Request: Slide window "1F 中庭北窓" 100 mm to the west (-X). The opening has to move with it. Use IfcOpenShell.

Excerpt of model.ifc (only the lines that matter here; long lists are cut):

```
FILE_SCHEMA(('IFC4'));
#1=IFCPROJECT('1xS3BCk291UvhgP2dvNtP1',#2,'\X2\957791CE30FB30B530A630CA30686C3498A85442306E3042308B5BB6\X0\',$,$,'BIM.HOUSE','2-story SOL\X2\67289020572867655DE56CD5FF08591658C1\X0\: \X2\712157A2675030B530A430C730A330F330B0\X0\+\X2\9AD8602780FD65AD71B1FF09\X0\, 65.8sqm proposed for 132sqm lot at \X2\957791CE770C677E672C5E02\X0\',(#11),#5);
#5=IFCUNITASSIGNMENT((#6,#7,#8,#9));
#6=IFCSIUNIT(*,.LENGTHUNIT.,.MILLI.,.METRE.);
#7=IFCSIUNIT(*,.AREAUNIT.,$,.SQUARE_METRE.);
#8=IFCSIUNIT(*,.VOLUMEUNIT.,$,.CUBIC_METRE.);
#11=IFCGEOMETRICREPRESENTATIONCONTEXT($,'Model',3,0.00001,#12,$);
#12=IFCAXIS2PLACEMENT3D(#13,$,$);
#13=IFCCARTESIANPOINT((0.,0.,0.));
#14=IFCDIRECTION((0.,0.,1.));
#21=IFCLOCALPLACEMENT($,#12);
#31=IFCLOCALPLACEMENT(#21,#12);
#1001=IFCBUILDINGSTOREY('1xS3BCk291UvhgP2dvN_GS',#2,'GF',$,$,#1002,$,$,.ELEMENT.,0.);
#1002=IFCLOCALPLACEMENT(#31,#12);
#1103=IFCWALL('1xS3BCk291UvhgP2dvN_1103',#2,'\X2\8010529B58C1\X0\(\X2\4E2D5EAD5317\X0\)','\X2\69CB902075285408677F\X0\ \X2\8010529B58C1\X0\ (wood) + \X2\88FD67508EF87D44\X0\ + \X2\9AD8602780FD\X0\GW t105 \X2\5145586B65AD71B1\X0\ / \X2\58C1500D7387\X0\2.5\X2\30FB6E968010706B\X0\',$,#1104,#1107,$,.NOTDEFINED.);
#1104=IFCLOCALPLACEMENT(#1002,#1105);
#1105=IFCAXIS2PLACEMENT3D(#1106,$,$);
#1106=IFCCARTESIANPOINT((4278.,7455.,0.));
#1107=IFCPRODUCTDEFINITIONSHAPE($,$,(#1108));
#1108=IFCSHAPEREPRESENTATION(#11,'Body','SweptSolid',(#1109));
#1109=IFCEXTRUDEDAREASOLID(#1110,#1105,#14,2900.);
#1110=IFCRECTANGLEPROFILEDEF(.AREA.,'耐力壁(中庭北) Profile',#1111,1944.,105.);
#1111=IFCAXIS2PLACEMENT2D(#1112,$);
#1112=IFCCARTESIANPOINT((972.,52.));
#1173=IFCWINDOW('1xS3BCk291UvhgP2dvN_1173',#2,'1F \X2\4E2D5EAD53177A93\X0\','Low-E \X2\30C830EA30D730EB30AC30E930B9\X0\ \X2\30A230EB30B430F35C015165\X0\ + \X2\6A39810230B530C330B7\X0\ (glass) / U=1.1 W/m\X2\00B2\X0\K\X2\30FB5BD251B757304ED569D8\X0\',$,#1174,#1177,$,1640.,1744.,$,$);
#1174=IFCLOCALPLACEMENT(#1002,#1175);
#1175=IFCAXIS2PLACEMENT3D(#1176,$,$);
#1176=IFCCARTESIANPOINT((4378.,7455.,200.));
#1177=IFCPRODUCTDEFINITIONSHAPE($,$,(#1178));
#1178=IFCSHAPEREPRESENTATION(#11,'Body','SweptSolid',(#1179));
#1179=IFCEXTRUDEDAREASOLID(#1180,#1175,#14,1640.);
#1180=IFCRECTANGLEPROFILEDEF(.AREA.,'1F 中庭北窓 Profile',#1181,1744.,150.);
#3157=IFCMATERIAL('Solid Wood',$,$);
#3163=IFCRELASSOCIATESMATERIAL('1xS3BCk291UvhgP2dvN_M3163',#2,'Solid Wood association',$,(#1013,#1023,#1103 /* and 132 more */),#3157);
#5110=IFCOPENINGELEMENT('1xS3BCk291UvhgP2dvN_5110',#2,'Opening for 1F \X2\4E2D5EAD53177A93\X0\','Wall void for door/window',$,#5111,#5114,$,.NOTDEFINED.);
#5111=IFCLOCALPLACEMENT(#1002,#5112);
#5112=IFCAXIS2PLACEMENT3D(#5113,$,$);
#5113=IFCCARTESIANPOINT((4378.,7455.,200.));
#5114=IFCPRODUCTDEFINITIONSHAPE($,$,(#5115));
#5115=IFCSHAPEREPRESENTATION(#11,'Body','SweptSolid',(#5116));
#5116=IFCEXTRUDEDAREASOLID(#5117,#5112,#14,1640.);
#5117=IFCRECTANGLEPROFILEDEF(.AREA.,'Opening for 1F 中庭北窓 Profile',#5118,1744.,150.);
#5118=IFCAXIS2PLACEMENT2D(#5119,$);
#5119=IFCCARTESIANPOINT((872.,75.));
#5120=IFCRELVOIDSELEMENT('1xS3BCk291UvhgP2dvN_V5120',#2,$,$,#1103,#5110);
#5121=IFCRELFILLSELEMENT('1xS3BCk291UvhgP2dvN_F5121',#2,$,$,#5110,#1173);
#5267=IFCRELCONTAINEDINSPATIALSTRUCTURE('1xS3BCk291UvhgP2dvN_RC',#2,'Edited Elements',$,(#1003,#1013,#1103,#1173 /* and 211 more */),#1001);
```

```python
import ifcopenshell
import ifcopenshell.api.geometry
import ifcopenshell.util.placement

model = ifcopenshell.open("model.ifc")

window = model.by_id(1173)
opening = window.FillsVoids[0].RelatingOpeningElement
wall = opening.VoidsElements[0].RelatingBuildingElement

wall_matrix = ifcopenshell.util.placement.get_local_placement(wall.ObjectPlacement)
shift = wall_matrix[:3, 0] * -100.0
before = ifcopenshell.util.placement.get_local_placement(window.ObjectPlacement)[:3, 3].copy()

# The window is not placed relative to its opening, so move both.
for product in (opening, window):
    matrix = ifcopenshell.util.placement.get_local_placement(product.ObjectPlacement)
    matrix[:3, 3] += shift
    ifcopenshell.api.geometry.edit_object_placement(model, product=product, matrix=matrix, is_si=False)

after = ifcopenshell.util.placement.get_local_placement(window.ObjectPlacement)[:3, 3]
print("window moved by", (after - before).round(3) + 0.0)

model.write("model_v2.ifc")
```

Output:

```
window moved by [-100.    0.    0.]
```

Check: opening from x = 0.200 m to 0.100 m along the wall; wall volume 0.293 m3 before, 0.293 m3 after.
